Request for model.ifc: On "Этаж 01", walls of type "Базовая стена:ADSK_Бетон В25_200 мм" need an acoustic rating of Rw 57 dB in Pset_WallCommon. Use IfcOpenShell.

First a look at what the model holds.

```python
import ifcopenshell
import ifcopenshell.util.element

model = ifcopenshell.open("model.ifc")
print(model.schema)
storey = next(s for s in model.by_type("IfcBuildingStorey") if s.Name == "Этаж 01")
walls = [e for e in ifcopenshell.util.element.get_decomposition(storey) if e.is_a("IfcWall")]
seen = {}
for e in walls:
    element_type = ifcopenshell.util.element.get_type(e)
    key = (element_type.Name if element_type != e and element_type else None, ifcopenshell.util.element.get_pset(e, "Pset_WallCommon", "AcousticRating"))
    seen[key] = seen.get(key, 0) + 1
for (name, value), count in sorted(seen.items(), key=str):
    print(count, "x", name, "|", value)
```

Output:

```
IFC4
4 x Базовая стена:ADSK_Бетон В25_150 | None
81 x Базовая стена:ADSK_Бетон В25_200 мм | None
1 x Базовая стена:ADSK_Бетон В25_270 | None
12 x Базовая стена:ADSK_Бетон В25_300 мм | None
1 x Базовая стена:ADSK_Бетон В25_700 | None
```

```python
import ifcopenshell
import ifcopenshell.api.pset
import ifcopenshell.util.element

model = ifcopenshell.open("model.ifc")

storey = next(s for s in model.by_type("IfcBuildingStorey") if s.Name == "Этаж 01")
walls = [e for e in ifcopenshell.util.element.get_decomposition(storey) if e.is_a("IfcWall")]

count = 0
for e in walls:
    element_type = ifcopenshell.util.element.get_type(e)
    if element_type in (None, e) or element_type.Name != "Базовая стена:ADSK_Бетон В25_200 мм":
        continue
    # add_pset returns the element's existing set when there is one.
    pset = ifcopenshell.api.pset.add_pset(model, product=e, name="Pset_WallCommon")
    ifcopenshell.api.pset.edit_pset(model, pset=pset, properties={"AcousticRating": "Rw 57 dB"})
    count += 1

print(count, "walls updated")

model.write("model-out.ifc")
```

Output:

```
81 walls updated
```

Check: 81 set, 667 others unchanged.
